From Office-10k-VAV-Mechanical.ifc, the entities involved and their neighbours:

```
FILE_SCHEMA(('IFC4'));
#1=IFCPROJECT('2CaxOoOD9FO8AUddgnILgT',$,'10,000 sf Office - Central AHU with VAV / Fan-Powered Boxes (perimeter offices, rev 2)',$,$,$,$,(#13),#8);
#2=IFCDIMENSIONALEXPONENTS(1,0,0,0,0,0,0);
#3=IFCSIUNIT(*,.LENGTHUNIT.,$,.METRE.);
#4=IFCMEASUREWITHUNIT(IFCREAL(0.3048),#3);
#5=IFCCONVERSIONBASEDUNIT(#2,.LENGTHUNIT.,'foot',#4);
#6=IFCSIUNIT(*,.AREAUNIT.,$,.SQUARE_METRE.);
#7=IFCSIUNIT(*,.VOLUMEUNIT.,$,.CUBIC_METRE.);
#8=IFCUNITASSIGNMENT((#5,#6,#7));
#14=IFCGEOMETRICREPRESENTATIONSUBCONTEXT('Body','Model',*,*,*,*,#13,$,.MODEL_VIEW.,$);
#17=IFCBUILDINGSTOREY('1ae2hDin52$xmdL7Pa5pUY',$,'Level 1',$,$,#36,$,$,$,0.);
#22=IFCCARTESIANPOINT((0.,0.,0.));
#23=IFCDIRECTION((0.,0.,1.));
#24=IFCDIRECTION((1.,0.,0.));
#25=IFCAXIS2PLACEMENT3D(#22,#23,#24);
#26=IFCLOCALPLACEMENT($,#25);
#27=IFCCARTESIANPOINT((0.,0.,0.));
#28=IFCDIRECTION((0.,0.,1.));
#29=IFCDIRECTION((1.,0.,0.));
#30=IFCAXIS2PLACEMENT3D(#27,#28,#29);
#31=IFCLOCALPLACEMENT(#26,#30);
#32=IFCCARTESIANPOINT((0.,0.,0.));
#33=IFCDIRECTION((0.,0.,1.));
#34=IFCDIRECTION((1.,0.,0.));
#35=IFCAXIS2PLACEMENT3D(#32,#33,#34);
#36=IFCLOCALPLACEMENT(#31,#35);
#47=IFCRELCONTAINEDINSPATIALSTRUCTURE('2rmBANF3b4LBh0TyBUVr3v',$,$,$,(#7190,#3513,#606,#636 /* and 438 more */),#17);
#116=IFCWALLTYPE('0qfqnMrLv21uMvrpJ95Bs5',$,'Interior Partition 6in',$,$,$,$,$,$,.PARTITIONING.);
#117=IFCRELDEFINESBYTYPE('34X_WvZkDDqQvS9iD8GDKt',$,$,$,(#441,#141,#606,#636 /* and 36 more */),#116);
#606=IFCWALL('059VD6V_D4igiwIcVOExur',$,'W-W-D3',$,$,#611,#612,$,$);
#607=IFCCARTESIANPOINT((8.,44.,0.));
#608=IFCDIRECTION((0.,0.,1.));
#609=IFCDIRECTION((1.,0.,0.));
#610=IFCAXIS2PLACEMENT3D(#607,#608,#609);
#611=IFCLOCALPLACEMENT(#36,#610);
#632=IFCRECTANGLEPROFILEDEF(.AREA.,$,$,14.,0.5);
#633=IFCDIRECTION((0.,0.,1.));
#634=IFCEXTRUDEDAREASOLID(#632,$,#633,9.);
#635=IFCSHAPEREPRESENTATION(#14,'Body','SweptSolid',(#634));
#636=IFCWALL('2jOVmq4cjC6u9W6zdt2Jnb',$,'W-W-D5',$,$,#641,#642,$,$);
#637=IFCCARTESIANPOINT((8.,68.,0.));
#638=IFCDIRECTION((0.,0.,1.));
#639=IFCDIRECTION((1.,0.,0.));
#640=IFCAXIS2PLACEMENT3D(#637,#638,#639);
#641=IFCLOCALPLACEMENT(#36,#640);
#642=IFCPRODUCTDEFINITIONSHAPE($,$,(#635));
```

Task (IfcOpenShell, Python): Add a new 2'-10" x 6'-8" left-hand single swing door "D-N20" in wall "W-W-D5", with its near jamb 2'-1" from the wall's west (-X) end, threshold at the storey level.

```python
import numpy as np
import ifcopenshell
import ifcopenshell.api.feature
import ifcopenshell.api.geometry
import ifcopenshell.api.root
import ifcopenshell.api.spatial
import ifcopenshell.geom
import ifcopenshell.util.element
import ifcopenshell.util.placement
import ifcopenshell.util.representation
import ifcopenshell.util.shape
import ifcopenshell.util.unit

model = ifcopenshell.open("Office-10k-VAV-Mechanical.ifc")
unit_scale = ifcopenshell.util.unit.calculate_unit_scale(model)
settings = ifcopenshell.geom.settings()


def volume(element):
    """Net volume in cubic metres, openings subtracted."""
    shape = ifcopenshell.geom.create_shape(settings, element)
    return ifcopenshell.util.shape.get_volume(shape.geometry)


wall = model.by_guid("2jOVmq4cjC6u9W6zdt2Jnb")
storey = ifcopenshell.util.element.get_container(wall, ifc_class="IfcBuildingStorey")
context = ifcopenshell.util.representation.get_context(model, "Model", "Body", "MODEL_VIEW")
before = volume(wall)

width, height, from_end, sill = 0.8636, 2.032, 0.635, 0.0  # metres

# The wall runs along its own X axis, and the end named is its -X end.
wall_shape = ifcopenshell.geom.create_shape(settings, wall)
x, y, z = ifcopenshell.util.shape.get_vertices(wall_shape.geometry).T
start = x.min() + from_end
face, thickness = float(y.min()), float(y.max() - y.min())
wall_matrix = ifcopenshell.util.placement.get_local_placement(wall.ObjectPlacement)
level = ifcopenshell.util.placement.get_local_placement(storey.ObjectPlacement)[2, 3]


def in_wall(x, y):
    """Placement at x, y metres in the wall's axes, at sill height."""
    matrix = wall_matrix.copy()
    matrix[:, 3] = wall_matrix @ np.array([x / unit_scale, y / unit_scale, 0.0, 1.0])
    matrix[2, 3] = level + sill / unit_scale
    return matrix


# Opening: a box that overshoots both wall faces by 50 mm.
opening = ifcopenshell.api.root.create_entity(model, ifc_class="IfcOpeningElement", predefined_type="OPENING")
box = ifcopenshell.api.geometry.add_wall_representation(
    model, context=context, length=width, height=height, thickness=thickness + 0.1
)
ifcopenshell.api.geometry.assign_representation(model, product=opening, representation=box)
ifcopenshell.api.geometry.edit_object_placement(model, product=opening, matrix=in_wall(start, face - 0.05), is_si=False)
ifcopenshell.api.feature.add_feature(model, feature=opening, element=wall)

door = ifcopenshell.api.root.create_entity(model, ifc_class="IfcDoor", name="D-N20", predefined_type="DOOR")
door.OverallWidth, door.OverallHeight = width / unit_scale, height / unit_scale
door.OperationType = "SINGLE_SWING_LEFT"
body = ifcopenshell.api.geometry.add_door_representation(
    model,
    context=context,
    overall_width=door.OverallWidth,
    overall_height=door.OverallHeight,
    operation_type="SINGLE_SWING_LEFT",
    lining_properties={"LiningDepth": thickness / unit_scale, "ThresholdDepth": thickness / unit_scale},
)
ifcopenshell.api.geometry.assign_representation(model, product=door, representation=body)
ifcopenshell.api.spatial.assign_container(model, products=[door], relating_structure=storey)
ifcopenshell.api.feature.add_filling(model, opening=opening, element=door)

# The lining spans the wall, so the door starts at the wall face.
ifcopenshell.api.geometry.edit_object_placement(model, product=door, matrix=in_wall(start, face), is_si=False)

after = volume(wall)

print(f"wall volume {before:.3f} -> {after:.3f} m3")

model.write("Office-10k-VAV-Mechanical_edited.ifc")
```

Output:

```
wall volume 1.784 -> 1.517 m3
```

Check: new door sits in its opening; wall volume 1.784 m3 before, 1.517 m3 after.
